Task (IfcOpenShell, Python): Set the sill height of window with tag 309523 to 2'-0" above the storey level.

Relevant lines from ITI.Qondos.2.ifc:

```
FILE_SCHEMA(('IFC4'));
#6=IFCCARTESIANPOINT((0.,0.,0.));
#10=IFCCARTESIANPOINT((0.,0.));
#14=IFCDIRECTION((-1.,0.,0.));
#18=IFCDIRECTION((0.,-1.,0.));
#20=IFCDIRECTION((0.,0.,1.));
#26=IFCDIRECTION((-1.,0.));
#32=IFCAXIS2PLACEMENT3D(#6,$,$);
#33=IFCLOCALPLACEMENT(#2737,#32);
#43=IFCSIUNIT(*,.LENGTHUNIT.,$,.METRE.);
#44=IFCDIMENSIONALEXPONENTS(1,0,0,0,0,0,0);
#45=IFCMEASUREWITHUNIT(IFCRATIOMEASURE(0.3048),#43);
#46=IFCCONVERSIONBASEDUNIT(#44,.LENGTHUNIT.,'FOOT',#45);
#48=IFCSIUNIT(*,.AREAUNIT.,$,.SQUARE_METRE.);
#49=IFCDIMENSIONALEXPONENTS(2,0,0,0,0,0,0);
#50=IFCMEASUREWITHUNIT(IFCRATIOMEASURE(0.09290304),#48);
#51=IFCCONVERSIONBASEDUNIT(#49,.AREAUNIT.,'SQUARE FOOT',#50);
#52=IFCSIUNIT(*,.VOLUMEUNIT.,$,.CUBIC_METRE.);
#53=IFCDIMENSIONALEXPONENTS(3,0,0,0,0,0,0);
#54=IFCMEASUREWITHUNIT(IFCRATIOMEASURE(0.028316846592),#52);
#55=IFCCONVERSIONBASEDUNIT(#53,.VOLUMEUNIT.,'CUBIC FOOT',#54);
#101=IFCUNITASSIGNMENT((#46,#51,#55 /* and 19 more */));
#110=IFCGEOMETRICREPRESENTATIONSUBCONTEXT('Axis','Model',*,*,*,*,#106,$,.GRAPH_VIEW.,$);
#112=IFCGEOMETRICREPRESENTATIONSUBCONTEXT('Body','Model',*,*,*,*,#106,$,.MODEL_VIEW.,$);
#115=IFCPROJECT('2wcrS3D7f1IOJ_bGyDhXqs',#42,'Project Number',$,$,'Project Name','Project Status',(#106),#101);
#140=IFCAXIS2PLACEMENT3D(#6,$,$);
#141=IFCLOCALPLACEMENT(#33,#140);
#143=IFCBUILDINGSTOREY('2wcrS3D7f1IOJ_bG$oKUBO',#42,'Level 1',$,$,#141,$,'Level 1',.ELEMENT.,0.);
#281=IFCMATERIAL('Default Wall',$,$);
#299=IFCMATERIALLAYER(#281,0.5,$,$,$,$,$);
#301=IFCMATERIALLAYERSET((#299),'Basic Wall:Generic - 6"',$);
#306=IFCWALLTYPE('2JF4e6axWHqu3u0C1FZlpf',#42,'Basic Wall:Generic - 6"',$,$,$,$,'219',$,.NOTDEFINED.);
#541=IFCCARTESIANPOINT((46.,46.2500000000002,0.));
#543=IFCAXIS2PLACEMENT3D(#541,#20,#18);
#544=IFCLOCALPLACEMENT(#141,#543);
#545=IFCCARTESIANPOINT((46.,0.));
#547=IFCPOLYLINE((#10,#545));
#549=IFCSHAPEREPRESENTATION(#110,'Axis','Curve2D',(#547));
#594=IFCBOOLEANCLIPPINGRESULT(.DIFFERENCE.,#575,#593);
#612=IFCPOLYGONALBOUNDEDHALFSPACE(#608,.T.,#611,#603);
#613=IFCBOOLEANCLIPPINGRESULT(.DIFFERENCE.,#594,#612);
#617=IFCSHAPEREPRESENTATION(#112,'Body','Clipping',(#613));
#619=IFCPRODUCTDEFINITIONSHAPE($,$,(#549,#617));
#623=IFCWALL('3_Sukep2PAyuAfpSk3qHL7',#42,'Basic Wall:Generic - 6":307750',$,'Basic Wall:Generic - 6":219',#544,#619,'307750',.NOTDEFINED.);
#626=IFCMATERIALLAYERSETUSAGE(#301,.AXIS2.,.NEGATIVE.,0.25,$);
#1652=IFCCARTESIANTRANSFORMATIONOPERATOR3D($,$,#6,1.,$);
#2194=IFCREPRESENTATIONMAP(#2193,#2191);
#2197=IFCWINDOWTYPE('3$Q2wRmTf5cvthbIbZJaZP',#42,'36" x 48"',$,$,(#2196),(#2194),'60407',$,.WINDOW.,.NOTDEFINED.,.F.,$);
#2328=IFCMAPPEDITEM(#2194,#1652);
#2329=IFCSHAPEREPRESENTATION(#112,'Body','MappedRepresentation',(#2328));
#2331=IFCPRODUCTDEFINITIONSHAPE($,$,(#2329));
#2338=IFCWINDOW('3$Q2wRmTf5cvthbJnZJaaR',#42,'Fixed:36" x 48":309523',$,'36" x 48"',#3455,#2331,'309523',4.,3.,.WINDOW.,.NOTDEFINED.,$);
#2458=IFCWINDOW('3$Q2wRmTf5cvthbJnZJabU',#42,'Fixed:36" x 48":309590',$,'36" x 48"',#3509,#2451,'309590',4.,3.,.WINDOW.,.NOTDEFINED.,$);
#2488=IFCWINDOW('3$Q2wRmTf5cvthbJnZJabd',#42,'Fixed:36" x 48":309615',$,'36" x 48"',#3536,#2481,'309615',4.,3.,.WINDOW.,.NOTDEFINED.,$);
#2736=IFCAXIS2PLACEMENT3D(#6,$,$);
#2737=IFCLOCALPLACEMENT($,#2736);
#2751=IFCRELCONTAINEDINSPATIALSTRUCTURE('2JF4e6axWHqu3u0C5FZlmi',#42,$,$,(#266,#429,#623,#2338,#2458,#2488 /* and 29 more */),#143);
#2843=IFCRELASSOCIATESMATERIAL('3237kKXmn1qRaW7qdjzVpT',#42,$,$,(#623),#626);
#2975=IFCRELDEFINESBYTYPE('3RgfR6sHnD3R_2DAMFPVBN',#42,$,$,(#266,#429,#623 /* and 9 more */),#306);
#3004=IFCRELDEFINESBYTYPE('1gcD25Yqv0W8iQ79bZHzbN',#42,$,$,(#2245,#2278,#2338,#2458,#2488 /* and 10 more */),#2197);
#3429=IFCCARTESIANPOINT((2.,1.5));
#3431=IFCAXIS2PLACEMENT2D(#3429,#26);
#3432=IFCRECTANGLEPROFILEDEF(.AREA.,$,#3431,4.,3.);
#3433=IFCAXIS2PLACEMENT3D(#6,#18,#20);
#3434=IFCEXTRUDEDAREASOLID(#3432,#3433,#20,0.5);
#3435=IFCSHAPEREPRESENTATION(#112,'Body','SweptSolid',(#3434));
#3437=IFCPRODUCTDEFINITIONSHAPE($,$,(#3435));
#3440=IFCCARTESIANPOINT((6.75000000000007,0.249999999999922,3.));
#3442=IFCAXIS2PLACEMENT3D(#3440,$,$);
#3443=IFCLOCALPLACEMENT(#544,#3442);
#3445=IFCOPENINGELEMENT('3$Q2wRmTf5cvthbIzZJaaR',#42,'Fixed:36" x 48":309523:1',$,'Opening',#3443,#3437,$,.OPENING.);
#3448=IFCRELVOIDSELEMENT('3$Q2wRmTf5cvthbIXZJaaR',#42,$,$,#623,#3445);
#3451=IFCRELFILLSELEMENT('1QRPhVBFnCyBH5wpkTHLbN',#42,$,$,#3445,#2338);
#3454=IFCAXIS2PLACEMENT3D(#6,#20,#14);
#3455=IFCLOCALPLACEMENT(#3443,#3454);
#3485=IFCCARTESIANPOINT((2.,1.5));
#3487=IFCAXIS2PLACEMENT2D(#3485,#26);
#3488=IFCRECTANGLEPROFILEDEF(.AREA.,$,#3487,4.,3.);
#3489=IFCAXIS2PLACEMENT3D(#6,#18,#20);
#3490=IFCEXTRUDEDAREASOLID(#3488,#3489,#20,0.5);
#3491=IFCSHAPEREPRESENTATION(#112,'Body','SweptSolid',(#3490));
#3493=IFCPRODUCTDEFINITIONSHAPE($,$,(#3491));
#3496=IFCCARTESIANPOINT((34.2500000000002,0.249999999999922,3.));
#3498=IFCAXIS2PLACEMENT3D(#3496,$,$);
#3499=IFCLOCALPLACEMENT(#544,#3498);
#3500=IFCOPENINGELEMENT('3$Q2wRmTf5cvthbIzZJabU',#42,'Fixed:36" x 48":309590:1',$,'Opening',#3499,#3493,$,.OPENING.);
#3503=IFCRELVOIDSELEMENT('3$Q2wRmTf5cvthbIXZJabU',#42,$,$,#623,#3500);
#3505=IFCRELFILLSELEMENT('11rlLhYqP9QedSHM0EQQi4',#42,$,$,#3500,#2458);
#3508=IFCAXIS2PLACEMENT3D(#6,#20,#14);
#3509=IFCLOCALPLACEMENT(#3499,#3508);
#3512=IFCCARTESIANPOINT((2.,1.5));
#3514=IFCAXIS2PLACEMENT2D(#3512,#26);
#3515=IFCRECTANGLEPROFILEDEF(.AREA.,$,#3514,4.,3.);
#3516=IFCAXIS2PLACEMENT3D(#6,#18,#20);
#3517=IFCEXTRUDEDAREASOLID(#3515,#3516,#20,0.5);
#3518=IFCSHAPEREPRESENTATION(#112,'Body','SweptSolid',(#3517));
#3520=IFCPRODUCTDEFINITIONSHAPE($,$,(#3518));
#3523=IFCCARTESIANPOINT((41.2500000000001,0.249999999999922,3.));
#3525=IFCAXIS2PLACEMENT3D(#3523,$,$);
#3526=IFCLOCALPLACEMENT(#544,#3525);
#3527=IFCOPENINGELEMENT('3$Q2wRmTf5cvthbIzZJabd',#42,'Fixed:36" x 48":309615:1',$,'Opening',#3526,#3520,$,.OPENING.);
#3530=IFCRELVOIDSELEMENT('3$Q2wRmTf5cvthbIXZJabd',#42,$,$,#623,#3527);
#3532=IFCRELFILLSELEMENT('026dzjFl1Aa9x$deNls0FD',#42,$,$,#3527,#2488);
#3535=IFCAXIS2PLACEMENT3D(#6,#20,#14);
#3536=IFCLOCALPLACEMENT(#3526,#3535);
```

```python
import numpy as np
import ifcopenshell
import ifcopenshell.api.geometry
import ifcopenshell.geom
import ifcopenshell.util.element
import ifcopenshell.util.placement
import ifcopenshell.util.shape
import ifcopenshell.util.unit

model = ifcopenshell.open("ITI.Qondos.2.ifc")
unit_scale = ifcopenshell.util.unit.calculate_unit_scale(model)

window = model.by_guid("3$Q2wRmTf5cvthbJnZJaaR")
opening = window.FillsVoids[0].RelatingOpeningElement
storey = ifcopenshell.util.element.get_container(window, ifc_class="IfcBuildingStorey")
level = ifcopenshell.util.placement.get_local_placement(storey.ObjectPlacement)[2, 3]

# The opening's origin need not be at the sill, so measure its lowest point.
shape = ifcopenshell.geom.create_shape(ifcopenshell.geom.settings(), opening)
bottom = ifcopenshell.util.shape.get_shape_bottom_elevation(shape, shape.geometry) / unit_scale
dz = level + 24 * 0.0254 / unit_scale - bottom

shift = np.array([0.0, 0.0, dz])
# The window is placed relative to its opening, so it follows when the opening moves.
matrix = ifcopenshell.util.placement.get_local_placement(opening.ObjectPlacement)
matrix[:3, 3] += shift
ifcopenshell.api.geometry.edit_object_placement(
    model, product=opening, matrix=matrix, is_si=False, should_transform_children=True
)

print(f"moved by {dz * unit_scale:+.3f} m")

model.write("ITI.Qondos.2_rev.ifc")
```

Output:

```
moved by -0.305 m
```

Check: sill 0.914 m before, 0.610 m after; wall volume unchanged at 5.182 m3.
